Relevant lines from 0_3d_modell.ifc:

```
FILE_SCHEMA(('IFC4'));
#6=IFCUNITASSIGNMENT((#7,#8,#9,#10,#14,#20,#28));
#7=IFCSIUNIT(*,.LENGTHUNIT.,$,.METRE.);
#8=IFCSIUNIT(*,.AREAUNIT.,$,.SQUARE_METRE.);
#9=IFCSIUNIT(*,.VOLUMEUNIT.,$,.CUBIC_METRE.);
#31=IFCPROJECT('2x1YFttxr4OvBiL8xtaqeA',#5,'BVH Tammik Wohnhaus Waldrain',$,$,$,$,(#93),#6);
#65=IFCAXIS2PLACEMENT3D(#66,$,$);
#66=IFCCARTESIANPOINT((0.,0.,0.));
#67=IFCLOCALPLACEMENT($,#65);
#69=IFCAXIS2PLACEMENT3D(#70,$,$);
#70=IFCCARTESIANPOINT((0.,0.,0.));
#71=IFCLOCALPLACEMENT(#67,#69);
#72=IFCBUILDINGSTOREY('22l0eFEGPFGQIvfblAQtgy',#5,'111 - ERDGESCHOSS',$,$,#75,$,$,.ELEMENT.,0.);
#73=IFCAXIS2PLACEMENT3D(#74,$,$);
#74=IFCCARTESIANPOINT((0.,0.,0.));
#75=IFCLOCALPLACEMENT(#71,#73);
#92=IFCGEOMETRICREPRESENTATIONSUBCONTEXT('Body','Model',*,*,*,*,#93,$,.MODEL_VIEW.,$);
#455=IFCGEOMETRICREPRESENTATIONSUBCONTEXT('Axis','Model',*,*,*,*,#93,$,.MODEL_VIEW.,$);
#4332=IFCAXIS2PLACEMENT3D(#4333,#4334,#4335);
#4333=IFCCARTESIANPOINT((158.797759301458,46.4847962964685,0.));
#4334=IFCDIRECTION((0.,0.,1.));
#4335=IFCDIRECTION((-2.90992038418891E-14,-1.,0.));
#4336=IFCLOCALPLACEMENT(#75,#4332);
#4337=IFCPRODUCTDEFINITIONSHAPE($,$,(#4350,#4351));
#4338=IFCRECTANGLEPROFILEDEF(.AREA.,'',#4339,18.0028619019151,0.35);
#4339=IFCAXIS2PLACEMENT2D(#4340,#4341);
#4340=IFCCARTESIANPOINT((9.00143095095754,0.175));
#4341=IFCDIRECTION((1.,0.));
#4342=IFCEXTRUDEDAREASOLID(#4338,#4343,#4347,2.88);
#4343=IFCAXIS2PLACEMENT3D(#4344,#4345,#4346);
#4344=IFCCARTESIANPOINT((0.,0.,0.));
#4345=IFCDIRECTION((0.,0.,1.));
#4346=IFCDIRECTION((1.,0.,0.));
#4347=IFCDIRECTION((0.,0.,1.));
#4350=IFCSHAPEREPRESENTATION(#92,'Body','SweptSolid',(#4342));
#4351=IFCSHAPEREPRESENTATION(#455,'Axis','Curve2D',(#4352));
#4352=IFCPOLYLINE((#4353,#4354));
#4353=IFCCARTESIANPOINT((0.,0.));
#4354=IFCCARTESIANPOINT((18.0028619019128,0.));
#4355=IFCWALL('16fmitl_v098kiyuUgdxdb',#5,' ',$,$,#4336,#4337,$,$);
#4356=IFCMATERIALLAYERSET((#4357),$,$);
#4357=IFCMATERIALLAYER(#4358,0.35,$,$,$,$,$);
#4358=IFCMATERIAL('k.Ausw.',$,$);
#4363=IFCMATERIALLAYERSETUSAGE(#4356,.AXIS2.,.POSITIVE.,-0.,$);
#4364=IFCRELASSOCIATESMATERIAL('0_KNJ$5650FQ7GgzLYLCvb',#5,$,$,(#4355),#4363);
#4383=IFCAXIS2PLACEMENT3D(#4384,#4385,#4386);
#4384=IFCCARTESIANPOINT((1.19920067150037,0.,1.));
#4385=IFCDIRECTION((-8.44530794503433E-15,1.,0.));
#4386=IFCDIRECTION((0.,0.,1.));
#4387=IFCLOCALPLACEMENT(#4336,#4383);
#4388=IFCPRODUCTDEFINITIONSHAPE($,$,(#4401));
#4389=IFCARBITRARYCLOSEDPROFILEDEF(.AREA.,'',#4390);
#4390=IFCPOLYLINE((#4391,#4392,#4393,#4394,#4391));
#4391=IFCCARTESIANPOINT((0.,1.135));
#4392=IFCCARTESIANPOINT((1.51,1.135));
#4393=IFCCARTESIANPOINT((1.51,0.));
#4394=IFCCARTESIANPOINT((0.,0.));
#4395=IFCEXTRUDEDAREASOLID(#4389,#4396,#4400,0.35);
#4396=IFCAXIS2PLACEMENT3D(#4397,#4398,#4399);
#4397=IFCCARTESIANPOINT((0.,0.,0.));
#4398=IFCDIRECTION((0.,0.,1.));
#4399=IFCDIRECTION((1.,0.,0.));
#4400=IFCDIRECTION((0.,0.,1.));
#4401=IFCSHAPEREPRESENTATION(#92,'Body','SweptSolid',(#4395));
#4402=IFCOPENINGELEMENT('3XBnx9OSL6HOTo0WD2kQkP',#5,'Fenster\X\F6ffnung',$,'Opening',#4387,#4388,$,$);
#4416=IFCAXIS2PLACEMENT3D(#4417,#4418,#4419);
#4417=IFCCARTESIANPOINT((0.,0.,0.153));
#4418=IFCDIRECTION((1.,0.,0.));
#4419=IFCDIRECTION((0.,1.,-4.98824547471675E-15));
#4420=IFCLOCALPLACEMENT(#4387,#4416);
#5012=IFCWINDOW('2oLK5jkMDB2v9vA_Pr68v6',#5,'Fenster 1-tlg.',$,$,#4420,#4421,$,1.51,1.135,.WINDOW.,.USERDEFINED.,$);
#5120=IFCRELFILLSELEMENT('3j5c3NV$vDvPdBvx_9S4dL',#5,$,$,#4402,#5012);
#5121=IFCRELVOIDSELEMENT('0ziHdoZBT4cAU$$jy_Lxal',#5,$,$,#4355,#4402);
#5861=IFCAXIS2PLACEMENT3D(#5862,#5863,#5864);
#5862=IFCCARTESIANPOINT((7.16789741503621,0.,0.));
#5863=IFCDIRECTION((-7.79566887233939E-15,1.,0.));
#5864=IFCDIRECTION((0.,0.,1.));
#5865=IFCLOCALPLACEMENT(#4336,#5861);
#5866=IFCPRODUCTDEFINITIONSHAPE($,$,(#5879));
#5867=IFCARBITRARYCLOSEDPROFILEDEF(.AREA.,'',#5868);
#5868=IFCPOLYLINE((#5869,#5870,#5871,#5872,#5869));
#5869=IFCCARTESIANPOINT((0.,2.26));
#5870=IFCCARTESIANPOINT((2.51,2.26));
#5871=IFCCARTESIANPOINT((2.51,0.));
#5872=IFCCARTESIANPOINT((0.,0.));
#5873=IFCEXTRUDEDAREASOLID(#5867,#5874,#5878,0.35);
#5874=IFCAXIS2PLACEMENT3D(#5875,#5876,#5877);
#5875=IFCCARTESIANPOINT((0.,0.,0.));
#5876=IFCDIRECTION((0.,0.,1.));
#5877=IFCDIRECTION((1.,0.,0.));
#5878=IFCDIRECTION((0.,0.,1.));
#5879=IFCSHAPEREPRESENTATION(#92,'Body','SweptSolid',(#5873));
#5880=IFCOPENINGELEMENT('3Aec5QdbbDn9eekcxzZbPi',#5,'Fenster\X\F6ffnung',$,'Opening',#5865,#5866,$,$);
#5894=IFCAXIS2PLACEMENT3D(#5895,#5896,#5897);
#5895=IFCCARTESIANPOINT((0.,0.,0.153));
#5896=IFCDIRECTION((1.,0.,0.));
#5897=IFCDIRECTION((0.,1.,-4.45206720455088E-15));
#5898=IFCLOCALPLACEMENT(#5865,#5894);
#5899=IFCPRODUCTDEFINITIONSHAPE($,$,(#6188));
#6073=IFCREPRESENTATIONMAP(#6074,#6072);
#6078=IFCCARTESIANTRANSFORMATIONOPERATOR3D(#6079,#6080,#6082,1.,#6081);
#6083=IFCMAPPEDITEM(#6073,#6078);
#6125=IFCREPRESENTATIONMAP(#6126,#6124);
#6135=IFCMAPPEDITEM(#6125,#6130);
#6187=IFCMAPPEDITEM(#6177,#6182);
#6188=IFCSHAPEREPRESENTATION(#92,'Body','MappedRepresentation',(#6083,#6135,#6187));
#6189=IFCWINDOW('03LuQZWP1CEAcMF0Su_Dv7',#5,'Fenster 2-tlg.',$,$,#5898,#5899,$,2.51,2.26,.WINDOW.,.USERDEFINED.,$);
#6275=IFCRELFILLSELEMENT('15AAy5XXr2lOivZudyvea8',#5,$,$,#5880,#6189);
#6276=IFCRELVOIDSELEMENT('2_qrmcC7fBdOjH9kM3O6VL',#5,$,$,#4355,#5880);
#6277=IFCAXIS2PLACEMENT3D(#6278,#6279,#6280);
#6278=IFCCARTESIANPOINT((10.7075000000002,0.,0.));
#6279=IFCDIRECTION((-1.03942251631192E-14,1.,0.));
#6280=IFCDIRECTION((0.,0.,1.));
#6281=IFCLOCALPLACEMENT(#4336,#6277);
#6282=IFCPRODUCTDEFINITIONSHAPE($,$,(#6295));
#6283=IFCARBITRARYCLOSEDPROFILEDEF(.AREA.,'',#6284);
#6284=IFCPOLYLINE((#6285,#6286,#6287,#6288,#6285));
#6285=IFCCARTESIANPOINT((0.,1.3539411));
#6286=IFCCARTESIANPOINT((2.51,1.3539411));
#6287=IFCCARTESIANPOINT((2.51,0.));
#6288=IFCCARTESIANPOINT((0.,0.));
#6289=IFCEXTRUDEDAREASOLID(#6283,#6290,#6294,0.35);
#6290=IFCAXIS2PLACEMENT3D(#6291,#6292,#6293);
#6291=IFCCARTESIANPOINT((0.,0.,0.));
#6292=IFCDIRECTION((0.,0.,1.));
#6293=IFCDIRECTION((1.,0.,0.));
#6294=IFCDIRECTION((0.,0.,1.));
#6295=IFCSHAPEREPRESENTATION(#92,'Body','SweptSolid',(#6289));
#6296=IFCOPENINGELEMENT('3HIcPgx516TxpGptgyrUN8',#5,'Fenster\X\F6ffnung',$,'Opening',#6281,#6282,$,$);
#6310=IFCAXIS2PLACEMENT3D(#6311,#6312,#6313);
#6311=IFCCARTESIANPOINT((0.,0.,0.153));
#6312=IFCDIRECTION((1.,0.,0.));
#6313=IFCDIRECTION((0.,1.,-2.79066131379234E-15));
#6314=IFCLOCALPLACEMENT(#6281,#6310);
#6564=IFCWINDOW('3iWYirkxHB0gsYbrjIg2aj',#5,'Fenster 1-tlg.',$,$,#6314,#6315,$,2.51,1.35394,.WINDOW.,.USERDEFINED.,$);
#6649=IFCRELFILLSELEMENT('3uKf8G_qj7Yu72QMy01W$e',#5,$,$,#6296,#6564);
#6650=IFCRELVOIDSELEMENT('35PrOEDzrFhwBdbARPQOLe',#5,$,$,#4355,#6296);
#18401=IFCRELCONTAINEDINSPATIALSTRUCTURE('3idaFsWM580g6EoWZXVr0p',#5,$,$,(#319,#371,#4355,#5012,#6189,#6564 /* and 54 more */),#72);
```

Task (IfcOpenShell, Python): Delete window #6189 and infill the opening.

```python
import ifcopenshell
import ifcopenshell.api.feature
import ifcopenshell.api.root
import ifcopenshell.geom
import ifcopenshell.util.shape

model = ifcopenshell.open("0_3d_modell.ifc")
settings = ifcopenshell.geom.settings()


def volume(element):
    """Net volume in cubic metres, openings subtracted."""
    shape = ifcopenshell.geom.create_shape(settings, element)
    return ifcopenshell.util.shape.get_volume(shape.geometry)


window = model.by_guid("03LuQZWP1CEAcMF0Su_Dv7")
opening = window.FillsVoids[0].RelatingOpeningElement
wall = opening.VoidsElements[0].RelatingBuildingElement
before = volume(wall)

ifcopenshell.api.root.remove_product(model, product=window)
ifcopenshell.api.feature.remove_feature(model, feature=opening)

after = volume(wall)

print(f"wall volume {before:.3f} -> {after:.3f} m3")

model.write("0_3d_modell_rev.ifc")
```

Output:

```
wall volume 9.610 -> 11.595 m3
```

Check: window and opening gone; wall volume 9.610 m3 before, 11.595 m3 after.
